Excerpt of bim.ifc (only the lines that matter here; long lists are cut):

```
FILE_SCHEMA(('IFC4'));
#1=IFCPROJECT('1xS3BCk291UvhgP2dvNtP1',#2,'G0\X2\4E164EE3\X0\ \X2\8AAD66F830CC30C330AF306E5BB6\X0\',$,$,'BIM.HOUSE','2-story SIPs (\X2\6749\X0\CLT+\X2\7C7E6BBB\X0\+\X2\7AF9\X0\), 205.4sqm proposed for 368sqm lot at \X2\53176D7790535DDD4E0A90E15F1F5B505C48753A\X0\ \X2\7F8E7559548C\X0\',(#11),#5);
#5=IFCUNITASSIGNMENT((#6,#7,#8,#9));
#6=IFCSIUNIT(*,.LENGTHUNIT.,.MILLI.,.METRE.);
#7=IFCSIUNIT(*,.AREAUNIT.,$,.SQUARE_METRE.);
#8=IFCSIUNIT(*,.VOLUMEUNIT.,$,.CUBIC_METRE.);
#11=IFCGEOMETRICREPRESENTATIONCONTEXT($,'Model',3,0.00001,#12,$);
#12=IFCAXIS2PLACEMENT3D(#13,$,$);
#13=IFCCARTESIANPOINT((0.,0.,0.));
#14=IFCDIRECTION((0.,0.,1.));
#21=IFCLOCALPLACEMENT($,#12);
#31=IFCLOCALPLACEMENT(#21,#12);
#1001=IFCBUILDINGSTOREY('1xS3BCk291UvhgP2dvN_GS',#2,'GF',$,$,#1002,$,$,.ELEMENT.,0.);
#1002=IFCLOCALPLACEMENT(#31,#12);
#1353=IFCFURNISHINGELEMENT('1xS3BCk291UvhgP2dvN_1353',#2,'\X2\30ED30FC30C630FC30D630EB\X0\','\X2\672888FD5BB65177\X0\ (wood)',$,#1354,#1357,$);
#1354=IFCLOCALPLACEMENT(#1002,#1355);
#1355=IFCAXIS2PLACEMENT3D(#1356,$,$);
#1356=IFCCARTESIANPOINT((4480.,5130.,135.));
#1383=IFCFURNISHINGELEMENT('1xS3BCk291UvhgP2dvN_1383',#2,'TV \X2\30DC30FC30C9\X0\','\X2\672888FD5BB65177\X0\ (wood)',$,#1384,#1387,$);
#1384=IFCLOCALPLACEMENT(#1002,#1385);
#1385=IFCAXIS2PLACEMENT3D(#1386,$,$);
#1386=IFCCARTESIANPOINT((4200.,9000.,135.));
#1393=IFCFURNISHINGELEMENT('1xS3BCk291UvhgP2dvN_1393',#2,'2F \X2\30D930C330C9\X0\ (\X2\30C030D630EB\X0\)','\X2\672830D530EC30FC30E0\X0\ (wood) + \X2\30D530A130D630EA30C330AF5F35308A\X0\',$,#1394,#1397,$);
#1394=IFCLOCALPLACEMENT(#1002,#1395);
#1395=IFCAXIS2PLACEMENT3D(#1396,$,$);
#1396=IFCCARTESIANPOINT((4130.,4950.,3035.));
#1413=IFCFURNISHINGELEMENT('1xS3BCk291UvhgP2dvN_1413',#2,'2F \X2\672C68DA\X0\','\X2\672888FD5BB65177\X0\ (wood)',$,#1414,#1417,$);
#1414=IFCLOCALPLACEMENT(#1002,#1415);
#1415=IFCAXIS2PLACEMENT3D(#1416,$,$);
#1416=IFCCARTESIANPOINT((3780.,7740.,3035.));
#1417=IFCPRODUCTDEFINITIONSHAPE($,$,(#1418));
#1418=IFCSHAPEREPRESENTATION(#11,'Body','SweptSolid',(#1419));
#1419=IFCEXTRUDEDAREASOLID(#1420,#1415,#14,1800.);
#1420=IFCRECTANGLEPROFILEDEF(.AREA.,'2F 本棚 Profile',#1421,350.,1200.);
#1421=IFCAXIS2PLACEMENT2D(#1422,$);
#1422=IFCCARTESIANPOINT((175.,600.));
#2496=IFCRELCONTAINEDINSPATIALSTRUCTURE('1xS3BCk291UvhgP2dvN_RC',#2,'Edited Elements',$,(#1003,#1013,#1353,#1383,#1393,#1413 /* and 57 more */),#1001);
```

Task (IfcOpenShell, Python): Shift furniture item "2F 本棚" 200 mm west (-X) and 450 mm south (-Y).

```python
import ifcopenshell
import ifcopenshell.api.geometry
import ifcopenshell.util.placement
import ifcopenshell.util.unit

model = ifcopenshell.open("bim.ifc")
unit_scale = ifcopenshell.util.unit.calculate_unit_scale(model)

item = model.by_guid("1xS3BCk291UvhgP2dvN_1413")
matrix = ifcopenshell.util.placement.get_local_placement(item.ObjectPlacement)
matrix[0, 3] -= 0.2 / unit_scale
matrix[1, 3] -= 0.45 / unit_scale
ifcopenshell.api.geometry.edit_object_placement(model, product=item, matrix=matrix, is_si=False)

print(ifcopenshell.util.placement.get_local_placement(item.ObjectPlacement).round(3) + 0.0)

model.write("bim_updated.ifc")
```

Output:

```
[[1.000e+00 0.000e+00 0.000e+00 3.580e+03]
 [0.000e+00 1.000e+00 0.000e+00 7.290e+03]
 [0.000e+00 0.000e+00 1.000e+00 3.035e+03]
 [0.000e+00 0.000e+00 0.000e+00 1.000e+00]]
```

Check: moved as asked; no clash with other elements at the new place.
